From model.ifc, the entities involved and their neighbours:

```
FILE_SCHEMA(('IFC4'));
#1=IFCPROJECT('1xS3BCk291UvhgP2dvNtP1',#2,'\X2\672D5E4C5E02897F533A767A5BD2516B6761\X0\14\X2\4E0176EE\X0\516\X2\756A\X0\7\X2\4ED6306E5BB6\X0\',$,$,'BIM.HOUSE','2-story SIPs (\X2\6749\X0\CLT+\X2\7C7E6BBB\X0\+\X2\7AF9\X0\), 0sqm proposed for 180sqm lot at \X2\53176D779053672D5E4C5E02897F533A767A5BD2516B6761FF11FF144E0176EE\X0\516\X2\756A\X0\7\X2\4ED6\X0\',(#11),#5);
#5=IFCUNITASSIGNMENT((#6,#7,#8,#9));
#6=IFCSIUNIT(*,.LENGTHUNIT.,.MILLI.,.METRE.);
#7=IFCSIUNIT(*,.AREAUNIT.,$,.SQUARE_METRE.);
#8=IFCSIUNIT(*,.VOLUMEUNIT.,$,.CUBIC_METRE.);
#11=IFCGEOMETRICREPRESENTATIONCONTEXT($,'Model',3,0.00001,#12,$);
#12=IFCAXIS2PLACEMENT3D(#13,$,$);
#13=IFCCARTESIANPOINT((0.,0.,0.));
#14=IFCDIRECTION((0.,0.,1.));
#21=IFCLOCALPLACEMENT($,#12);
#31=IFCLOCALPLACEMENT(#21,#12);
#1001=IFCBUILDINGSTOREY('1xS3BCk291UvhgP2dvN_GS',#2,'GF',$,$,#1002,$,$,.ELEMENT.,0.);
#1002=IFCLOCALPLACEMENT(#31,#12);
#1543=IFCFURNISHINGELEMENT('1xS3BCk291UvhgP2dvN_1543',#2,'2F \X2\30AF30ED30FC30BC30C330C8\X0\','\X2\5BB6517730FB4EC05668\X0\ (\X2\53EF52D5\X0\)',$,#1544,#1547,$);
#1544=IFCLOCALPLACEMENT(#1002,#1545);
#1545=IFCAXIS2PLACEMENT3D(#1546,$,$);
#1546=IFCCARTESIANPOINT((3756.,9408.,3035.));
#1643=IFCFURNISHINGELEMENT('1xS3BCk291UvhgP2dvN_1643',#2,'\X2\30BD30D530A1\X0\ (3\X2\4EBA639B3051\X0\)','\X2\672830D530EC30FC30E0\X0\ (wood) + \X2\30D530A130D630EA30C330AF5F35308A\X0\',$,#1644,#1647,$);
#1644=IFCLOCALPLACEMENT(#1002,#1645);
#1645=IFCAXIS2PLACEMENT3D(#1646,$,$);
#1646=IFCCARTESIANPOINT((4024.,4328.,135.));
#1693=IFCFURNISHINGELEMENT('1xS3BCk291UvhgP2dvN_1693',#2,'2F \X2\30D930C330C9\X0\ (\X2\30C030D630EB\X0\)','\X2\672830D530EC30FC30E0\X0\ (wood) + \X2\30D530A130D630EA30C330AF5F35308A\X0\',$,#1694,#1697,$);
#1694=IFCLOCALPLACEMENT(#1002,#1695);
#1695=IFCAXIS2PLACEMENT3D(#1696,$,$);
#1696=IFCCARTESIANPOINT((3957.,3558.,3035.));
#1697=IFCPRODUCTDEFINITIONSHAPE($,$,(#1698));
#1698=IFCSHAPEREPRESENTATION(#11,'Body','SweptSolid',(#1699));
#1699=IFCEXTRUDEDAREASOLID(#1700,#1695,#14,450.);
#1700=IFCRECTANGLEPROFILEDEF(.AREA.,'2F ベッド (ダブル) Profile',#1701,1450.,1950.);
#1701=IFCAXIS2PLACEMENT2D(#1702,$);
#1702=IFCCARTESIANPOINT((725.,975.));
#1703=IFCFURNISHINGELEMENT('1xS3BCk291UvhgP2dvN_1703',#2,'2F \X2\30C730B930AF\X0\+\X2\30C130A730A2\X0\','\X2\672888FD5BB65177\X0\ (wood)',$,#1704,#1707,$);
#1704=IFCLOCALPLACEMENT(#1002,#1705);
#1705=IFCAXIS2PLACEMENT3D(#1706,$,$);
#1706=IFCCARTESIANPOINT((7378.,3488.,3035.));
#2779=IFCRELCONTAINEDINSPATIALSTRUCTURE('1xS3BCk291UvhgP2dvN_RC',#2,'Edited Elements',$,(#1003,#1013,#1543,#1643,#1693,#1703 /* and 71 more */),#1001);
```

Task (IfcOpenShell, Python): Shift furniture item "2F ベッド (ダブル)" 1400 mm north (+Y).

```python
import ifcopenshell
import ifcopenshell.api.geometry
import ifcopenshell.util.placement
import ifcopenshell.util.unit

model = ifcopenshell.open("model.ifc")
unit_scale = ifcopenshell.util.unit.calculate_unit_scale(model)

item = model.by_guid("1xS3BCk291UvhgP2dvN_1693")
matrix = ifcopenshell.util.placement.get_local_placement(item.ObjectPlacement)
matrix[1, 3] += 1.4 / unit_scale
ifcopenshell.api.geometry.edit_object_placement(model, product=item, matrix=matrix, is_si=False)

print(ifcopenshell.util.placement.get_local_placement(item.ObjectPlacement).round(3) + 0.0)

model.write("model_updated.ifc")
```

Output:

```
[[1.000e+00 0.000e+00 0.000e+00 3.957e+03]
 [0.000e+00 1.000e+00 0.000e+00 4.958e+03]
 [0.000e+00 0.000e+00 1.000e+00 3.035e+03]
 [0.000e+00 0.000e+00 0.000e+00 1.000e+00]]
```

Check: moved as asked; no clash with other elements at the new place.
